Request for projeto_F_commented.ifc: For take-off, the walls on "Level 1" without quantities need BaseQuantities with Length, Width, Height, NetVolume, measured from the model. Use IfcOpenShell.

First a look at what the model holds.

```python
import ifcopenshell
import ifcopenshell.util.element
import ifcopenshell.util.unit

model = ifcopenshell.open("projeto_F_commented.ifc")
print(model.schema)
for unit_type in ("LENGTHUNIT", "AREAUNIT", "VOLUMEUNIT"):
    print(unit_type, ifcopenshell.util.unit.calculate_unit_scale(model, unit_type))
storey = next(s for s in model.by_type("IfcBuildingStorey") if s.Name == "Level 1")
walls = [e for e in ifcopenshell.util.element.get_decomposition(storey) if e.is_a("IfcWall")]
for e in sorted(walls, key=lambda e: e.id()):
    print(e.id(), e.is_a(), e.Name, list(ifcopenshell.util.element.get_psets(e, qtos_only=True)), sep=" | ")
```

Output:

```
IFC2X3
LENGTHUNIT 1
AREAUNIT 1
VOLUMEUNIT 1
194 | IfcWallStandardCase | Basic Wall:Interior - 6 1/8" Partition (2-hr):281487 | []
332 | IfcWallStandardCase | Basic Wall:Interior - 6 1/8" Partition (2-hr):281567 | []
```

```python
import ifcopenshell
import ifcopenshell.api.pset
import ifcopenshell.geom
import ifcopenshell.util.element
import ifcopenshell.util.shape
import ifcopenshell.util.unit

model = ifcopenshell.open("projeto_F_commented.ifc")
unit_scale = ifcopenshell.util.unit.calculate_unit_scale(model)
volume_scale = ifcopenshell.util.unit.calculate_unit_scale(model, "VOLUMEUNIT")
settings = ifcopenshell.geom.settings()

storey = next(s for s in model.by_type("IfcBuildingStorey") if s.Name == "Level 1")
walls = [e for e in ifcopenshell.util.element.get_decomposition(storey) if e.is_a("IfcWall")]

for e in sorted(walls, key=lambda e: e.id()):
    if ifcopenshell.util.element.get_psets(e, qtos_only=True, should_inherit=False):
        continue
    # Geometry comes back in metres, in the element's own axes.
    shape = ifcopenshell.geom.create_shape(settings, e)
    values = {
        "Length": ifcopenshell.util.shape.get_x(shape.geometry) / unit_scale,
        "Width": ifcopenshell.util.shape.get_y(shape.geometry) / unit_scale,
        "Height": ifcopenshell.util.shape.get_z(shape.geometry) / unit_scale,
        "NetVolume": ifcopenshell.util.shape.get_volume(shape.geometry) / volume_scale,
    }
    qto = ifcopenshell.api.pset.add_qto(model, product=e, name="BaseQuantities")
    ifcopenshell.api.pset.edit_qto(model, qto=qto, properties=values)
    print(e.id(), {k: round(v, 3) for k, v in values.items()})

model.write("projeto_F_commented_v2.ifc")
```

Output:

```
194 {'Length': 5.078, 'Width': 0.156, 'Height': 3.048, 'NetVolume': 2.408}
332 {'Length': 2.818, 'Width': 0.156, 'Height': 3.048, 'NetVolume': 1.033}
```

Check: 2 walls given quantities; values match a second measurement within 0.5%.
